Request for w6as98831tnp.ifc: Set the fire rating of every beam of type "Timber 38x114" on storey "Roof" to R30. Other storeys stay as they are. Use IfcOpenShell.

First a look at what the model holds.

```python
import ifcopenshell
import ifcopenshell.util.element

model = ifcopenshell.open("w6as98831tnp.ifc")
print(model.schema)
storey = next(s for s in model.by_type("IfcBuildingStorey") if s.Name == "Roof")
beams = [e for e in ifcopenshell.util.element.get_decomposition(storey) if e.is_a("IfcBeam")]
seen = {}
for e in beams:
    element_type = ifcopenshell.util.element.get_type(e)
    key = (element_type.Name if element_type != e and element_type else None, ifcopenshell.util.element.get_pset(e, "Pset_BeamCommon", "FireRating"))
    seen[key] = seen.get(key, 0) + 1
for (name, value), count in sorted(seen.items(), key=str):
    print(count, "x", name, "|", value)
```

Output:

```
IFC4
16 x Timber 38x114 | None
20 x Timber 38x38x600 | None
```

```python
import ifcopenshell
import ifcopenshell.api.pset
import ifcopenshell.util.element

model = ifcopenshell.open("w6as98831tnp.ifc")

storey = next(s for s in model.by_type("IfcBuildingStorey") if s.Name == "Roof")
beams = [e for e in ifcopenshell.util.element.get_decomposition(storey) if e.is_a("IfcBeam")]

count = 0
for e in beams:
    element_type = ifcopenshell.util.element.get_type(e)
    if element_type in (None, e) or element_type.Name != "Timber 38x114":
        continue
    # add_pset returns the element's existing set when there is one.
    pset = ifcopenshell.api.pset.add_pset(model, product=e, name="Pset_BeamCommon")
    ifcopenshell.api.pset.edit_pset(model, pset=pset, properties={"FireRating": "R30"})
    count += 1

print(count, "beams updated")

model.write("w6as98831tnp_rev.ifc")
```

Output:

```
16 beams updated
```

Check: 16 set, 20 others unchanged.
